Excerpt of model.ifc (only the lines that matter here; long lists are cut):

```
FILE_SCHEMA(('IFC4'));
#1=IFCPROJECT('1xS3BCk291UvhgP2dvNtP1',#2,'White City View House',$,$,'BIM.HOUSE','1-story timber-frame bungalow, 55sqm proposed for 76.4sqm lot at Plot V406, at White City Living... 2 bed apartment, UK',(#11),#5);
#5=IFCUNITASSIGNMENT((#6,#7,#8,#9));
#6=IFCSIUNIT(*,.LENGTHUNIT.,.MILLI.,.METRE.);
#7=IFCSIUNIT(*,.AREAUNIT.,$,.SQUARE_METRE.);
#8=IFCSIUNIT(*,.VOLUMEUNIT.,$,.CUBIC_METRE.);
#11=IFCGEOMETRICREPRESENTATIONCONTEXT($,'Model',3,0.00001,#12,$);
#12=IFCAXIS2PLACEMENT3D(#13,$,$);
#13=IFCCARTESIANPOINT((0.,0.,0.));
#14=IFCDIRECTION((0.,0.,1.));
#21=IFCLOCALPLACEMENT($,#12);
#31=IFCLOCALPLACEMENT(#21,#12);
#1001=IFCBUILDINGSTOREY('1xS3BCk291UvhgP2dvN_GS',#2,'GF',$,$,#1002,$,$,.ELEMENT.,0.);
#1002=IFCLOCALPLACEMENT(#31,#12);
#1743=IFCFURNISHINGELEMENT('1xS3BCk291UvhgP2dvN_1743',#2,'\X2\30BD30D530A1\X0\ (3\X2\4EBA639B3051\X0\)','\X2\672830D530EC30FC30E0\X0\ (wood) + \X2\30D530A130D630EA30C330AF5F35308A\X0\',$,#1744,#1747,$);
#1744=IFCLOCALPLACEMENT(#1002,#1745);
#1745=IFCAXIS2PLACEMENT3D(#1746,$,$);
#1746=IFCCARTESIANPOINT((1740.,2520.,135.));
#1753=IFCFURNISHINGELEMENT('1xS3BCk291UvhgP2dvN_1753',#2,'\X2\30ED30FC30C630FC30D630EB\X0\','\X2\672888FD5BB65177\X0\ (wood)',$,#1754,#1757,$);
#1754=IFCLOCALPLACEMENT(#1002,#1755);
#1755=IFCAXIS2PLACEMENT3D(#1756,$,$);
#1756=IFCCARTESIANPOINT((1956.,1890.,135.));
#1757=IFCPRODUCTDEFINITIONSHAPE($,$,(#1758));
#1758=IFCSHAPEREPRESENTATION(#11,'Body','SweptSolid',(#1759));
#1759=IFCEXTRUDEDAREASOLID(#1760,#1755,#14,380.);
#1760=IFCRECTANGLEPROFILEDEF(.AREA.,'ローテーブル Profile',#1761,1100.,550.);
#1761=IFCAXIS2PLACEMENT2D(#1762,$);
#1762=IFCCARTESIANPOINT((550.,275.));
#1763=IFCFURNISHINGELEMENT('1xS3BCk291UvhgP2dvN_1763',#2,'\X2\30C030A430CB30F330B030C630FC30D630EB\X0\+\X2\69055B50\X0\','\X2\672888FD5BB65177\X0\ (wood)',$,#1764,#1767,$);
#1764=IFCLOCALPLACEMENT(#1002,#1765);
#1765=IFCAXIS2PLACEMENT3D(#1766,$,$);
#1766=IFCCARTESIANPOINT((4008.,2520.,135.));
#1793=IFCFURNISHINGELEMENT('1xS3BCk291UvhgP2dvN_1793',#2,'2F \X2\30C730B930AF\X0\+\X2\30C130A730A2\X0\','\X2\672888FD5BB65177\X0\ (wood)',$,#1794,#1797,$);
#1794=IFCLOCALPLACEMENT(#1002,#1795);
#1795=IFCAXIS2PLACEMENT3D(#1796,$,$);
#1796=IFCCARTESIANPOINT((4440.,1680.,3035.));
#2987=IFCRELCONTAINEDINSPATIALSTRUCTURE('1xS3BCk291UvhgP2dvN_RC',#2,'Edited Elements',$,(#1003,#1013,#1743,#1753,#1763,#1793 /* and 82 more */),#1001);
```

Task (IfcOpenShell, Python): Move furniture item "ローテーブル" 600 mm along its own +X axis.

```python
import ifcopenshell
import ifcopenshell.api.geometry
import ifcopenshell.util.placement

model = ifcopenshell.open("model.ifc")

item = model.by_guid("1xS3BCk291UvhgP2dvN_1753")
matrix = ifcopenshell.util.placement.get_local_placement(item.ObjectPlacement)
matrix[:3, 3] += matrix[:3, 0] * 600.0
ifcopenshell.api.geometry.edit_object_placement(model, product=item, matrix=matrix, is_si=False)

print(ifcopenshell.util.placement.get_local_placement(item.ObjectPlacement).round(3) + 0.0)

model.write("model_rev.ifc")
```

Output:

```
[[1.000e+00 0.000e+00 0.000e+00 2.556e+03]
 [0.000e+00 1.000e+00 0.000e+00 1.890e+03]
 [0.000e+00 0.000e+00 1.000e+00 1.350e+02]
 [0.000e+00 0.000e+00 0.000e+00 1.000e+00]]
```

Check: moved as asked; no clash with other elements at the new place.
